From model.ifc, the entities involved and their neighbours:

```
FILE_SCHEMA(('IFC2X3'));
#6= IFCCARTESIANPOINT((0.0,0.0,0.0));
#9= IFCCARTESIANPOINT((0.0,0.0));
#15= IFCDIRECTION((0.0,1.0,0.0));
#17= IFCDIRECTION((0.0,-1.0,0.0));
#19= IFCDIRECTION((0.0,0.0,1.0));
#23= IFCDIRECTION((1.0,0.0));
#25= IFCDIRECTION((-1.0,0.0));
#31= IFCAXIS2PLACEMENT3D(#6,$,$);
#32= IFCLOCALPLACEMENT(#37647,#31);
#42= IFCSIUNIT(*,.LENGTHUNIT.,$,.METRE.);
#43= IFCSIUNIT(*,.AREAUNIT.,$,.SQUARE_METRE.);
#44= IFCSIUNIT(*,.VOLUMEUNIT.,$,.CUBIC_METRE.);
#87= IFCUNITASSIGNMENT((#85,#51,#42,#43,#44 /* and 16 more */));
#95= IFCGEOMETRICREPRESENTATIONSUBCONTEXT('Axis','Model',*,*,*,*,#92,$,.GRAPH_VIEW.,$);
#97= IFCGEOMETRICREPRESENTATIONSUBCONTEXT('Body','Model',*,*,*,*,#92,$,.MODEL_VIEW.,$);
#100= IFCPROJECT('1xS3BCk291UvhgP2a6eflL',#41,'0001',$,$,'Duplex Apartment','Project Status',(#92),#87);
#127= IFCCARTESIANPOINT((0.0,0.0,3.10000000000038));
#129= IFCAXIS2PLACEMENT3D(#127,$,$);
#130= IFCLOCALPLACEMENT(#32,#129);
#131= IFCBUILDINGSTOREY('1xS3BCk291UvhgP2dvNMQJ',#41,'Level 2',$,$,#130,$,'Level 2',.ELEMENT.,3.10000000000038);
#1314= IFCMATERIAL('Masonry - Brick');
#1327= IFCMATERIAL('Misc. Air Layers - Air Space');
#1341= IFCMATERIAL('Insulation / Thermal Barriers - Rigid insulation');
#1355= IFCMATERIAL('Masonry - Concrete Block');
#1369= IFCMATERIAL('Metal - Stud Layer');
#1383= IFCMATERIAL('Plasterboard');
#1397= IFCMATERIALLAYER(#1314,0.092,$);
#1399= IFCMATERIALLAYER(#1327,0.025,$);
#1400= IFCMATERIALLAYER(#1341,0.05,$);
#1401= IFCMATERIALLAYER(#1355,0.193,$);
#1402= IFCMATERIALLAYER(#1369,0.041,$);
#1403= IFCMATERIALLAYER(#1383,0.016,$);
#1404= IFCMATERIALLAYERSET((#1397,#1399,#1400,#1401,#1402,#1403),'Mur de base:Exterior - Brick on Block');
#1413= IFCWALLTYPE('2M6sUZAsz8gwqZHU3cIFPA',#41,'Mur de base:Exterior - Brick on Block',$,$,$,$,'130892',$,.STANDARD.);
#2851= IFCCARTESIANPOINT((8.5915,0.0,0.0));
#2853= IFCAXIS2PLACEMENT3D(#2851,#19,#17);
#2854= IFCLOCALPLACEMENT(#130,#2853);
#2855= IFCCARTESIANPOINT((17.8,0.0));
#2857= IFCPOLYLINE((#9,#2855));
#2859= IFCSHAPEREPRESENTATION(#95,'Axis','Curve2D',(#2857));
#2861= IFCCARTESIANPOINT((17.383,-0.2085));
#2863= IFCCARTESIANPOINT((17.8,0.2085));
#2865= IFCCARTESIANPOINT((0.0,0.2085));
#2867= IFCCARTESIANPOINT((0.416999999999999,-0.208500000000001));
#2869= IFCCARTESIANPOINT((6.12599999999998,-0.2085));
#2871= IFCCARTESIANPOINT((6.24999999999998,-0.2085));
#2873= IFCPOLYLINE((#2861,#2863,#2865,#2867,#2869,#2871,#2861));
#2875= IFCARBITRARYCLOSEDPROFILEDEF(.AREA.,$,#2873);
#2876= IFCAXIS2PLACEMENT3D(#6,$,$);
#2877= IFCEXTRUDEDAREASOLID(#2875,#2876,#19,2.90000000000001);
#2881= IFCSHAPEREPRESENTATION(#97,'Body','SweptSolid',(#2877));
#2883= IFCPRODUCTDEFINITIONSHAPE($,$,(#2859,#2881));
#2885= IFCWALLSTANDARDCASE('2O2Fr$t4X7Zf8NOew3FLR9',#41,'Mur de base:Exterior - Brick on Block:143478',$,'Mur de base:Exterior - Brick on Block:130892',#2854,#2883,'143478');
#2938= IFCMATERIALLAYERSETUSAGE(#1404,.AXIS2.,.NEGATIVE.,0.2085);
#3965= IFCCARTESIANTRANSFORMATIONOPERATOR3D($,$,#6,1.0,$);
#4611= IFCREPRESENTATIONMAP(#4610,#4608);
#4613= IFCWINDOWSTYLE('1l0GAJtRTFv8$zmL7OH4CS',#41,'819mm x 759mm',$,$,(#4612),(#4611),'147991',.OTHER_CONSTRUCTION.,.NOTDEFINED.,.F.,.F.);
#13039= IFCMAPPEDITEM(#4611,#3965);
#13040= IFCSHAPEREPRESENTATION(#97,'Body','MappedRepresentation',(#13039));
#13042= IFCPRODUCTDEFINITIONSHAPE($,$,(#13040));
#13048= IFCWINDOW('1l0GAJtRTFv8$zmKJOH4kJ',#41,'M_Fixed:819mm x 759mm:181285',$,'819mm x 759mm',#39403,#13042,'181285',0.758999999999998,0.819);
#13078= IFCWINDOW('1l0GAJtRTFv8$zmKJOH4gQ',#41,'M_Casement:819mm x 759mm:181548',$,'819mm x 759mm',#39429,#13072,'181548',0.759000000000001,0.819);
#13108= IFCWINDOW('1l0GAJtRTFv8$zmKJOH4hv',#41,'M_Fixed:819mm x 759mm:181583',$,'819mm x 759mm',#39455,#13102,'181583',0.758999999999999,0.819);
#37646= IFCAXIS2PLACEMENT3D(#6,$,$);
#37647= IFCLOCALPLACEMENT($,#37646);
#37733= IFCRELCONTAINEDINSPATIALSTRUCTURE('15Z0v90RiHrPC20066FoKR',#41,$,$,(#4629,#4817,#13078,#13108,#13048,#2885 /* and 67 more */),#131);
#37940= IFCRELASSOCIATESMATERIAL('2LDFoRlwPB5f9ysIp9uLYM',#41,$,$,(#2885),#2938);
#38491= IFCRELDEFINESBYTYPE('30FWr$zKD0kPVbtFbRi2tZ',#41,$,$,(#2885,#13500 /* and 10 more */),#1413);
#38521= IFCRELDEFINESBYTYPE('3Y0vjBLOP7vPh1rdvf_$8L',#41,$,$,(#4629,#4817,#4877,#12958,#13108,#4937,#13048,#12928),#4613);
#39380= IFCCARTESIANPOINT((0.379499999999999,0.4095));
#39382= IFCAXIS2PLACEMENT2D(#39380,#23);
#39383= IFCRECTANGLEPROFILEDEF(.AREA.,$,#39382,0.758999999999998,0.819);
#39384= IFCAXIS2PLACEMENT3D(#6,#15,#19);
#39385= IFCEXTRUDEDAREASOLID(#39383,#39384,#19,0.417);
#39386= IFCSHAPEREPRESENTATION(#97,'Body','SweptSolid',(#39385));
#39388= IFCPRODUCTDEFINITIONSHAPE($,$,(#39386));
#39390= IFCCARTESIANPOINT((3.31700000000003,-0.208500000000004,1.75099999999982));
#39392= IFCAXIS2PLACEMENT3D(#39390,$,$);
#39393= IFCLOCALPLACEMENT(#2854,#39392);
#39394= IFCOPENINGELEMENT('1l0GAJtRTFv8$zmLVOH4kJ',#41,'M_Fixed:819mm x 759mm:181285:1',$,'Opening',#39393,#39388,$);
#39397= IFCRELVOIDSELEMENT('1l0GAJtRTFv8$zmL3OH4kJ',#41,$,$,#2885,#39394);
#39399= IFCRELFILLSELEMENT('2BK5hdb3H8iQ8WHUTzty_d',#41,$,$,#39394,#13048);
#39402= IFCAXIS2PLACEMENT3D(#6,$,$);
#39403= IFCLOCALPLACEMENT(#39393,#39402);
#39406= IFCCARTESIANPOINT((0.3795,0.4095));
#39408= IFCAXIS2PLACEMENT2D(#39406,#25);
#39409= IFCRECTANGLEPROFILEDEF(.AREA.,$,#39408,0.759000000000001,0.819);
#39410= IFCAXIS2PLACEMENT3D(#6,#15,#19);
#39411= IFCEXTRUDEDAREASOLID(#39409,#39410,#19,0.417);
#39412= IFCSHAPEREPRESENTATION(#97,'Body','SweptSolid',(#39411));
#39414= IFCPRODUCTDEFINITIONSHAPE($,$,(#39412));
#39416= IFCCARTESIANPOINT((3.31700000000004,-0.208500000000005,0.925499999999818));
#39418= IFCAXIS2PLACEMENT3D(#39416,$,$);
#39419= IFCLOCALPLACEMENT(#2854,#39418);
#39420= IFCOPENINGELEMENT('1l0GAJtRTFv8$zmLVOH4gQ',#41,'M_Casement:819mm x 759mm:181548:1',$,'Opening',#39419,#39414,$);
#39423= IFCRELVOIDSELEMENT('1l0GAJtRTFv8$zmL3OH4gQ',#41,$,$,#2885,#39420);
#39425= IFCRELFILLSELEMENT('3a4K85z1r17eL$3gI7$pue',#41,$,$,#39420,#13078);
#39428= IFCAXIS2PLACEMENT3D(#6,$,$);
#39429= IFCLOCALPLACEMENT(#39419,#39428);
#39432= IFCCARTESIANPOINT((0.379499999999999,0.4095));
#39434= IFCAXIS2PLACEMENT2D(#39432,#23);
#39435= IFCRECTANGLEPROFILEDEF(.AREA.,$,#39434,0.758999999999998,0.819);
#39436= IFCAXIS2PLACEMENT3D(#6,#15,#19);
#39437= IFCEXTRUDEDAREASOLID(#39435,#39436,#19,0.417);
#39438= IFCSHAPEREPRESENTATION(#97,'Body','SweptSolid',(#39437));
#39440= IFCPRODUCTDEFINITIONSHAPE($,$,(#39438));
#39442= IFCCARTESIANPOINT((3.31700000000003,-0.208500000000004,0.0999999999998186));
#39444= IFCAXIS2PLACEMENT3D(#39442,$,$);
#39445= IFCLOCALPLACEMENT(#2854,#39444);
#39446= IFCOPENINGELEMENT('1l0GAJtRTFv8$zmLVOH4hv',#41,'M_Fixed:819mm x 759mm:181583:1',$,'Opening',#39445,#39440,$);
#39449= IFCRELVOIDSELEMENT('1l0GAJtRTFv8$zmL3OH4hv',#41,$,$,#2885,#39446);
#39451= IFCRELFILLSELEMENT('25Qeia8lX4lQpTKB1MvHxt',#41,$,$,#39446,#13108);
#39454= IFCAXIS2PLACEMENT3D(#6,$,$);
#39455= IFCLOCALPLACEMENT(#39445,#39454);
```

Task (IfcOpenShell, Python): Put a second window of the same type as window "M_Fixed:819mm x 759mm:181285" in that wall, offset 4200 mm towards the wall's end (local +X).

```python
import ifcopenshell
import ifcopenshell.api.feature
import ifcopenshell.api.geometry
import ifcopenshell.api.root
import ifcopenshell.geom
import ifcopenshell.util.element
import ifcopenshell.util.placement
import ifcopenshell.util.shape
import ifcopenshell.util.unit

model = ifcopenshell.open("model.ifc")
unit_scale = ifcopenshell.util.unit.calculate_unit_scale(model)
settings = ifcopenshell.geom.settings()


def volume(element):
    """Net volume in cubic metres, openings subtracted."""
    shape = ifcopenshell.geom.create_shape(settings, element)
    return ifcopenshell.util.shape.get_volume(shape.geometry)


def reuse_history(source, copy):
    """copy_class also copies each property set's owner history, people and application; keep the originals."""
    for rel in copy.IsDefinedBy:
        if rel.is_a("IfcRelDefinesByProperties") and (history := rel.RelatingPropertyDefinition.OwnerHistory):
            rel.RelatingPropertyDefinition.OwnerHistory = source.OwnerHistory
            ifcopenshell.util.element.remove_deep2(model, history)


window = model.by_guid("1l0GAJtRTFv8$zmKJOH4kJ")
opening = window.FillsVoids[0].RelatingOpeningElement
wall = opening.VoidsElements[0].RelatingBuildingElement
before = volume(wall)
shift = ifcopenshell.util.placement.get_local_placement(wall.ObjectPlacement)[:3, 0] * 4.2 / unit_scale

# copy_class copies the void relationship, type, container and properties, but no geometry.
new_opening = ifcopenshell.api.root.copy_class(model, product=opening)
new_opening.Representation = ifcopenshell.util.element.copy_deep(
    model, opening.Representation, exclude=["IfcGeometricRepresentationContext", "IfcRepresentationMap"]
)
new_opening.Name = "M_Fixed:819mm x 759mm"
new_window = ifcopenshell.api.root.copy_class(model, product=window)
new_window.Representation = ifcopenshell.util.element.copy_deep(
    model, window.Representation, exclude=["IfcGeometricRepresentationContext", "IfcRepresentationMap"]
)
new_window.Name = "M_Fixed:819mm x 759mm"
new_window.Tag = None
reuse_history(window, new_window)
fills = ifcopenshell.api.feature.add_filling(model, opening=new_opening, element=new_window)
fills.OwnerHistory = new_window.OwnerHistory  # required in IFC2X3

for old, new in ((opening, new_opening), (window, new_window)):
    matrix = ifcopenshell.util.placement.get_local_placement(old.ObjectPlacement)
    matrix[:3, 3] += shift
    ifcopenshell.api.geometry.edit_object_placement(model, product=new, matrix=matrix, is_si=False)

after = volume(wall)

print(f"wall volume {before:.3f} -> {after:.3f} m3")

model.write("model_v2.ifc")
```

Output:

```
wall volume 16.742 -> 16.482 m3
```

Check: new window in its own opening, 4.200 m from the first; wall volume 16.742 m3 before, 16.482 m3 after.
